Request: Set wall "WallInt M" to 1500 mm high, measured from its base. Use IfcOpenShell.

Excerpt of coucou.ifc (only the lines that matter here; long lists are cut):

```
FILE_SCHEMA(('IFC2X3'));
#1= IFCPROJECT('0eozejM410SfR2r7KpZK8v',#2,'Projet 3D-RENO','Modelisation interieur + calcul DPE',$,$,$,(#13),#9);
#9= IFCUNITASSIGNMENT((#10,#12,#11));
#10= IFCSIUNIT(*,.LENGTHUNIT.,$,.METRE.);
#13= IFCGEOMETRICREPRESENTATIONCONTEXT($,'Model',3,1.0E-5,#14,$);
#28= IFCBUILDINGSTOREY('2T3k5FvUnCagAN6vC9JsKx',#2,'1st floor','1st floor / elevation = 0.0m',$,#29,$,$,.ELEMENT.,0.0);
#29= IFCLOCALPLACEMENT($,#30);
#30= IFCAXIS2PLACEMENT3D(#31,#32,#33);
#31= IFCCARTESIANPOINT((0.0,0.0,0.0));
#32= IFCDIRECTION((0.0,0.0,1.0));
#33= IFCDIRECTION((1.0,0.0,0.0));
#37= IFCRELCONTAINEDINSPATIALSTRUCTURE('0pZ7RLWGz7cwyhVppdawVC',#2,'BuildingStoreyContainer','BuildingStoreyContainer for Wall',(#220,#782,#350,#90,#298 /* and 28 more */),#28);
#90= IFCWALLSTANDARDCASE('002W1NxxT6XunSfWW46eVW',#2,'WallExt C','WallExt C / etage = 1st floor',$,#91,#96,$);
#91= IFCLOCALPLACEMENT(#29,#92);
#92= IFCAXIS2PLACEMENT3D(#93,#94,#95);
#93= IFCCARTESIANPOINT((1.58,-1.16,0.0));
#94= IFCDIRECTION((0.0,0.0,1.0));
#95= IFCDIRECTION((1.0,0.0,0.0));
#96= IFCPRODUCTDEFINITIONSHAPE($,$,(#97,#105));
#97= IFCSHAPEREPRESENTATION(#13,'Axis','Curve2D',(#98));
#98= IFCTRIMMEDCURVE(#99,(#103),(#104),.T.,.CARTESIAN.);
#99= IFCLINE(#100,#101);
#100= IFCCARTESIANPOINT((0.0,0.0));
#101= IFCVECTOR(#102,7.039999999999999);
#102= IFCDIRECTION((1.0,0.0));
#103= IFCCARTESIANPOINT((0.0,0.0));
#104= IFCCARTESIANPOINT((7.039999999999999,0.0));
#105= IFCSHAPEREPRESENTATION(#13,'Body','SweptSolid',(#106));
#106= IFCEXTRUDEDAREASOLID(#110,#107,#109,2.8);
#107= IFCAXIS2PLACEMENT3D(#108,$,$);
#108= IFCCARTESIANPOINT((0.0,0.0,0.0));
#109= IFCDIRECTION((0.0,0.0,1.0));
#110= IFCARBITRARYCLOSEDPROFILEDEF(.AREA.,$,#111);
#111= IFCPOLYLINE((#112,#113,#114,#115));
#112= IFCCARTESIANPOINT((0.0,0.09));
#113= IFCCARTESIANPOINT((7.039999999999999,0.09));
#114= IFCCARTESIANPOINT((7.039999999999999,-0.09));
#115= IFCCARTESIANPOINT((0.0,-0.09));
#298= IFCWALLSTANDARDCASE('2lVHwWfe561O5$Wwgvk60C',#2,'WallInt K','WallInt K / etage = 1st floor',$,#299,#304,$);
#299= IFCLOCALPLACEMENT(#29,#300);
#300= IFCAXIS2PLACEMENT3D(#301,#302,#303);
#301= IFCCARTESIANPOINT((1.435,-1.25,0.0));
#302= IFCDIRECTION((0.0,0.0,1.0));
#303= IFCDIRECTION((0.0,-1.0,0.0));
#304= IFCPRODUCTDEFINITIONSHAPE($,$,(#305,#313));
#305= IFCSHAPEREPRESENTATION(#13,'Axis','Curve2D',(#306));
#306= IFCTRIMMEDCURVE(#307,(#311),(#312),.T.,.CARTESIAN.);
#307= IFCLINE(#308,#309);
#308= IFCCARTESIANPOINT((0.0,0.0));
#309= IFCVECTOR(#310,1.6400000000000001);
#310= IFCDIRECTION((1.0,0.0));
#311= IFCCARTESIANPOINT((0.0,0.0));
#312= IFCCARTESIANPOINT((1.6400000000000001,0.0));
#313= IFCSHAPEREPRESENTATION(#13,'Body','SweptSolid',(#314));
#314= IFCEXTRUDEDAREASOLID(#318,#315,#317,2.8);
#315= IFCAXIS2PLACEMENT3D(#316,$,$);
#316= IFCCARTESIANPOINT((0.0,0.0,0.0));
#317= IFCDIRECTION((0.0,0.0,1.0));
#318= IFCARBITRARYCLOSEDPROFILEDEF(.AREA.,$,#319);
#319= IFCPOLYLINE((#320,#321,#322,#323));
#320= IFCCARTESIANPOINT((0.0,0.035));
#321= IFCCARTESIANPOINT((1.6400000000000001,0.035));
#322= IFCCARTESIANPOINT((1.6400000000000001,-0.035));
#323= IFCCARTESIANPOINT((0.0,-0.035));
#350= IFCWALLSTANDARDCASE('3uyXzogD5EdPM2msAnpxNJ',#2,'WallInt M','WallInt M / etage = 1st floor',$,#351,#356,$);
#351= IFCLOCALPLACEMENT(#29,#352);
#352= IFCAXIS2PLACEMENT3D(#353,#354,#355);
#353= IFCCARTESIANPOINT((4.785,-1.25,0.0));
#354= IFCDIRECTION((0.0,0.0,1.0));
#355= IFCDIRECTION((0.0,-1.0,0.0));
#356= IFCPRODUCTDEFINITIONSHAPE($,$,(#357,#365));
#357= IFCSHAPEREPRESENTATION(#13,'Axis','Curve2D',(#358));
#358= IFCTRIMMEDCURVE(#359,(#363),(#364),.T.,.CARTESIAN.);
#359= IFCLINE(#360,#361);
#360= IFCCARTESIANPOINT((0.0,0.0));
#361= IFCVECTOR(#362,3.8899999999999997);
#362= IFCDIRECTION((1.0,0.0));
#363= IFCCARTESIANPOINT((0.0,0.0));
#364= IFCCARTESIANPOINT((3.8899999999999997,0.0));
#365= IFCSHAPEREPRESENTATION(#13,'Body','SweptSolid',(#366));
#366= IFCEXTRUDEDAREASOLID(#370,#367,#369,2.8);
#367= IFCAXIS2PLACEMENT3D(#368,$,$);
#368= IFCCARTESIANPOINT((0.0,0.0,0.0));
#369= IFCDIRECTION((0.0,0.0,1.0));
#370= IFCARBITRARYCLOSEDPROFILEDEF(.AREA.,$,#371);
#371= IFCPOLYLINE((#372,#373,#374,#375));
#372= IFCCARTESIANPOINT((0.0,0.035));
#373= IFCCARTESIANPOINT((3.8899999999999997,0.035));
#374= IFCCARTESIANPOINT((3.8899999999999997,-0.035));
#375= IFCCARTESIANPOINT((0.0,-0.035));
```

```python
import ifcopenshell
import ifcopenshell.geom
import ifcopenshell.util.shape
import ifcopenshell.util.unit

model = ifcopenshell.open("coucou.ifc")
unit_scale = ifcopenshell.util.unit.calculate_unit_scale(model)
settings = ifcopenshell.geom.settings()


def volume(element):
    """Net volume in cubic metres, openings subtracted."""
    shape = ifcopenshell.geom.create_shape(settings, element)
    return ifcopenshell.util.shape.get_volume(shape.geometry)


wall = model.by_guid("3uyXzogD5EdPM2msAnpxNJ")
before = volume(wall)

body = next(r for r in wall.Representation.Representations if r.RepresentationIdentifier == "Body")
solid = body.Items[0]
old_height = solid.Depth
solid.Depth = 1.5 / unit_scale
after = volume(wall)

print(f"height {old_height:g} -> {solid.Depth:g}, volume {before:.3f} -> {after:.3f} m3")

model.write("coucou_v2.ifc")
```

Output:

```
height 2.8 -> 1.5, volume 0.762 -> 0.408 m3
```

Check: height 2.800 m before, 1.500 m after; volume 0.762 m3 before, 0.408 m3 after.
